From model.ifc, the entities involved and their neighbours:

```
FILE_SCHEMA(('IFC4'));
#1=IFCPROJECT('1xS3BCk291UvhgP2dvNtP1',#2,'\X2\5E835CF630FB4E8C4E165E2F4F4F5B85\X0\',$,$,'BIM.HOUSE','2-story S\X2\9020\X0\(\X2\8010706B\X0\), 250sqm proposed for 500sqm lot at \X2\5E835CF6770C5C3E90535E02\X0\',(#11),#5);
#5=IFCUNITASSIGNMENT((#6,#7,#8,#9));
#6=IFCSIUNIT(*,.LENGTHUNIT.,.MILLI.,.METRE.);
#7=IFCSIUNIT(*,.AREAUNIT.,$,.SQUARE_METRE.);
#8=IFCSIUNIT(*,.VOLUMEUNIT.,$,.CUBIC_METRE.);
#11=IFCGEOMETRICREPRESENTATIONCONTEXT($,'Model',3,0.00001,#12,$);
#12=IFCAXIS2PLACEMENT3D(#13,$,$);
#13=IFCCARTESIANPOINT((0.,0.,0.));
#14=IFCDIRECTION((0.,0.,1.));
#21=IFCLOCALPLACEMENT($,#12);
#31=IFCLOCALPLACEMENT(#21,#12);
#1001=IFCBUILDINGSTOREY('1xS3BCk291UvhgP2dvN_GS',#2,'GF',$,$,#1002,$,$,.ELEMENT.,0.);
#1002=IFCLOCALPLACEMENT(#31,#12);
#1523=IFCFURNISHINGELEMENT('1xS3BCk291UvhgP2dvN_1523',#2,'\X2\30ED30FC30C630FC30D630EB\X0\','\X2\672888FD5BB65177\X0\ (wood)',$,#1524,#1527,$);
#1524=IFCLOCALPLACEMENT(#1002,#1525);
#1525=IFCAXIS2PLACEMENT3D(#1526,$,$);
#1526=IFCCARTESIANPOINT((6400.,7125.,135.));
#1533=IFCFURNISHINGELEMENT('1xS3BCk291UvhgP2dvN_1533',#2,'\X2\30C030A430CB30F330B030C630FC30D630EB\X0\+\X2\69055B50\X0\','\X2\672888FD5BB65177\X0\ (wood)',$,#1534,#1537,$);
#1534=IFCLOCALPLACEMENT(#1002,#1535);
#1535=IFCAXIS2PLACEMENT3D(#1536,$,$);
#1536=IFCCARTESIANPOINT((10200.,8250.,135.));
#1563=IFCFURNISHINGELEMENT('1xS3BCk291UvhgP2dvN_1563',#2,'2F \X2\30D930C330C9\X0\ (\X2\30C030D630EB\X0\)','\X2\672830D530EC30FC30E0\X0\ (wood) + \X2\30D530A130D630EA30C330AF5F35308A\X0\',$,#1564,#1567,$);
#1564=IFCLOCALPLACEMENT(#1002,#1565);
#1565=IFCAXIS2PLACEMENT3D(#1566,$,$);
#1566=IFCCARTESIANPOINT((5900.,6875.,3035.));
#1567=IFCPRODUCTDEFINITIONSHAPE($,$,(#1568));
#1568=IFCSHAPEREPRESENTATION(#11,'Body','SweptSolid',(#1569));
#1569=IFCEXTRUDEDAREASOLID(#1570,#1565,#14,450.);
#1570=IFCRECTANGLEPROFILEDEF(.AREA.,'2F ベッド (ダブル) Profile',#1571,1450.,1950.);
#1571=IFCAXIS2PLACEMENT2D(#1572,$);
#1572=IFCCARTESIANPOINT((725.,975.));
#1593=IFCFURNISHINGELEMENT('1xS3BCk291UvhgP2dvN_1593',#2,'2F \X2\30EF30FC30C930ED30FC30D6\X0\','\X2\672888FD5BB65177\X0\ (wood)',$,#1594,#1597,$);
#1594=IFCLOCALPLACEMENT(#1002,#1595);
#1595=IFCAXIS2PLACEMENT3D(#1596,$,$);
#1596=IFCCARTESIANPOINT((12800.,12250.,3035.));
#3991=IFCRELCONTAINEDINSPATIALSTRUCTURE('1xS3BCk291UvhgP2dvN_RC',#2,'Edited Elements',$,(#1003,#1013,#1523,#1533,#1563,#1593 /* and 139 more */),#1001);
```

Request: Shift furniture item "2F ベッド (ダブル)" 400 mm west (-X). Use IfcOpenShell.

```python
import ifcopenshell
import ifcopenshell.api.geometry
import ifcopenshell.util.placement
import ifcopenshell.util.unit

model = ifcopenshell.open("model.ifc")
unit_scale = ifcopenshell.util.unit.calculate_unit_scale(model)

item = model.by_guid("1xS3BCk291UvhgP2dvN_1563")
matrix = ifcopenshell.util.placement.get_local_placement(item.ObjectPlacement)
matrix[0, 3] -= 0.4 / unit_scale
ifcopenshell.api.geometry.edit_object_placement(model, product=item, matrix=matrix, is_si=False)

print(ifcopenshell.util.placement.get_local_placement(item.ObjectPlacement).round(3) + 0.0)

model.write("model_v2.ifc")
```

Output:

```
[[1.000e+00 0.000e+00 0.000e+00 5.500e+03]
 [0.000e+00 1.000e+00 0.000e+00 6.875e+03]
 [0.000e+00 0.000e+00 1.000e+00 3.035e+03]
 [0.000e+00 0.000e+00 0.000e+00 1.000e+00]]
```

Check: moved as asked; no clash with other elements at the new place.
